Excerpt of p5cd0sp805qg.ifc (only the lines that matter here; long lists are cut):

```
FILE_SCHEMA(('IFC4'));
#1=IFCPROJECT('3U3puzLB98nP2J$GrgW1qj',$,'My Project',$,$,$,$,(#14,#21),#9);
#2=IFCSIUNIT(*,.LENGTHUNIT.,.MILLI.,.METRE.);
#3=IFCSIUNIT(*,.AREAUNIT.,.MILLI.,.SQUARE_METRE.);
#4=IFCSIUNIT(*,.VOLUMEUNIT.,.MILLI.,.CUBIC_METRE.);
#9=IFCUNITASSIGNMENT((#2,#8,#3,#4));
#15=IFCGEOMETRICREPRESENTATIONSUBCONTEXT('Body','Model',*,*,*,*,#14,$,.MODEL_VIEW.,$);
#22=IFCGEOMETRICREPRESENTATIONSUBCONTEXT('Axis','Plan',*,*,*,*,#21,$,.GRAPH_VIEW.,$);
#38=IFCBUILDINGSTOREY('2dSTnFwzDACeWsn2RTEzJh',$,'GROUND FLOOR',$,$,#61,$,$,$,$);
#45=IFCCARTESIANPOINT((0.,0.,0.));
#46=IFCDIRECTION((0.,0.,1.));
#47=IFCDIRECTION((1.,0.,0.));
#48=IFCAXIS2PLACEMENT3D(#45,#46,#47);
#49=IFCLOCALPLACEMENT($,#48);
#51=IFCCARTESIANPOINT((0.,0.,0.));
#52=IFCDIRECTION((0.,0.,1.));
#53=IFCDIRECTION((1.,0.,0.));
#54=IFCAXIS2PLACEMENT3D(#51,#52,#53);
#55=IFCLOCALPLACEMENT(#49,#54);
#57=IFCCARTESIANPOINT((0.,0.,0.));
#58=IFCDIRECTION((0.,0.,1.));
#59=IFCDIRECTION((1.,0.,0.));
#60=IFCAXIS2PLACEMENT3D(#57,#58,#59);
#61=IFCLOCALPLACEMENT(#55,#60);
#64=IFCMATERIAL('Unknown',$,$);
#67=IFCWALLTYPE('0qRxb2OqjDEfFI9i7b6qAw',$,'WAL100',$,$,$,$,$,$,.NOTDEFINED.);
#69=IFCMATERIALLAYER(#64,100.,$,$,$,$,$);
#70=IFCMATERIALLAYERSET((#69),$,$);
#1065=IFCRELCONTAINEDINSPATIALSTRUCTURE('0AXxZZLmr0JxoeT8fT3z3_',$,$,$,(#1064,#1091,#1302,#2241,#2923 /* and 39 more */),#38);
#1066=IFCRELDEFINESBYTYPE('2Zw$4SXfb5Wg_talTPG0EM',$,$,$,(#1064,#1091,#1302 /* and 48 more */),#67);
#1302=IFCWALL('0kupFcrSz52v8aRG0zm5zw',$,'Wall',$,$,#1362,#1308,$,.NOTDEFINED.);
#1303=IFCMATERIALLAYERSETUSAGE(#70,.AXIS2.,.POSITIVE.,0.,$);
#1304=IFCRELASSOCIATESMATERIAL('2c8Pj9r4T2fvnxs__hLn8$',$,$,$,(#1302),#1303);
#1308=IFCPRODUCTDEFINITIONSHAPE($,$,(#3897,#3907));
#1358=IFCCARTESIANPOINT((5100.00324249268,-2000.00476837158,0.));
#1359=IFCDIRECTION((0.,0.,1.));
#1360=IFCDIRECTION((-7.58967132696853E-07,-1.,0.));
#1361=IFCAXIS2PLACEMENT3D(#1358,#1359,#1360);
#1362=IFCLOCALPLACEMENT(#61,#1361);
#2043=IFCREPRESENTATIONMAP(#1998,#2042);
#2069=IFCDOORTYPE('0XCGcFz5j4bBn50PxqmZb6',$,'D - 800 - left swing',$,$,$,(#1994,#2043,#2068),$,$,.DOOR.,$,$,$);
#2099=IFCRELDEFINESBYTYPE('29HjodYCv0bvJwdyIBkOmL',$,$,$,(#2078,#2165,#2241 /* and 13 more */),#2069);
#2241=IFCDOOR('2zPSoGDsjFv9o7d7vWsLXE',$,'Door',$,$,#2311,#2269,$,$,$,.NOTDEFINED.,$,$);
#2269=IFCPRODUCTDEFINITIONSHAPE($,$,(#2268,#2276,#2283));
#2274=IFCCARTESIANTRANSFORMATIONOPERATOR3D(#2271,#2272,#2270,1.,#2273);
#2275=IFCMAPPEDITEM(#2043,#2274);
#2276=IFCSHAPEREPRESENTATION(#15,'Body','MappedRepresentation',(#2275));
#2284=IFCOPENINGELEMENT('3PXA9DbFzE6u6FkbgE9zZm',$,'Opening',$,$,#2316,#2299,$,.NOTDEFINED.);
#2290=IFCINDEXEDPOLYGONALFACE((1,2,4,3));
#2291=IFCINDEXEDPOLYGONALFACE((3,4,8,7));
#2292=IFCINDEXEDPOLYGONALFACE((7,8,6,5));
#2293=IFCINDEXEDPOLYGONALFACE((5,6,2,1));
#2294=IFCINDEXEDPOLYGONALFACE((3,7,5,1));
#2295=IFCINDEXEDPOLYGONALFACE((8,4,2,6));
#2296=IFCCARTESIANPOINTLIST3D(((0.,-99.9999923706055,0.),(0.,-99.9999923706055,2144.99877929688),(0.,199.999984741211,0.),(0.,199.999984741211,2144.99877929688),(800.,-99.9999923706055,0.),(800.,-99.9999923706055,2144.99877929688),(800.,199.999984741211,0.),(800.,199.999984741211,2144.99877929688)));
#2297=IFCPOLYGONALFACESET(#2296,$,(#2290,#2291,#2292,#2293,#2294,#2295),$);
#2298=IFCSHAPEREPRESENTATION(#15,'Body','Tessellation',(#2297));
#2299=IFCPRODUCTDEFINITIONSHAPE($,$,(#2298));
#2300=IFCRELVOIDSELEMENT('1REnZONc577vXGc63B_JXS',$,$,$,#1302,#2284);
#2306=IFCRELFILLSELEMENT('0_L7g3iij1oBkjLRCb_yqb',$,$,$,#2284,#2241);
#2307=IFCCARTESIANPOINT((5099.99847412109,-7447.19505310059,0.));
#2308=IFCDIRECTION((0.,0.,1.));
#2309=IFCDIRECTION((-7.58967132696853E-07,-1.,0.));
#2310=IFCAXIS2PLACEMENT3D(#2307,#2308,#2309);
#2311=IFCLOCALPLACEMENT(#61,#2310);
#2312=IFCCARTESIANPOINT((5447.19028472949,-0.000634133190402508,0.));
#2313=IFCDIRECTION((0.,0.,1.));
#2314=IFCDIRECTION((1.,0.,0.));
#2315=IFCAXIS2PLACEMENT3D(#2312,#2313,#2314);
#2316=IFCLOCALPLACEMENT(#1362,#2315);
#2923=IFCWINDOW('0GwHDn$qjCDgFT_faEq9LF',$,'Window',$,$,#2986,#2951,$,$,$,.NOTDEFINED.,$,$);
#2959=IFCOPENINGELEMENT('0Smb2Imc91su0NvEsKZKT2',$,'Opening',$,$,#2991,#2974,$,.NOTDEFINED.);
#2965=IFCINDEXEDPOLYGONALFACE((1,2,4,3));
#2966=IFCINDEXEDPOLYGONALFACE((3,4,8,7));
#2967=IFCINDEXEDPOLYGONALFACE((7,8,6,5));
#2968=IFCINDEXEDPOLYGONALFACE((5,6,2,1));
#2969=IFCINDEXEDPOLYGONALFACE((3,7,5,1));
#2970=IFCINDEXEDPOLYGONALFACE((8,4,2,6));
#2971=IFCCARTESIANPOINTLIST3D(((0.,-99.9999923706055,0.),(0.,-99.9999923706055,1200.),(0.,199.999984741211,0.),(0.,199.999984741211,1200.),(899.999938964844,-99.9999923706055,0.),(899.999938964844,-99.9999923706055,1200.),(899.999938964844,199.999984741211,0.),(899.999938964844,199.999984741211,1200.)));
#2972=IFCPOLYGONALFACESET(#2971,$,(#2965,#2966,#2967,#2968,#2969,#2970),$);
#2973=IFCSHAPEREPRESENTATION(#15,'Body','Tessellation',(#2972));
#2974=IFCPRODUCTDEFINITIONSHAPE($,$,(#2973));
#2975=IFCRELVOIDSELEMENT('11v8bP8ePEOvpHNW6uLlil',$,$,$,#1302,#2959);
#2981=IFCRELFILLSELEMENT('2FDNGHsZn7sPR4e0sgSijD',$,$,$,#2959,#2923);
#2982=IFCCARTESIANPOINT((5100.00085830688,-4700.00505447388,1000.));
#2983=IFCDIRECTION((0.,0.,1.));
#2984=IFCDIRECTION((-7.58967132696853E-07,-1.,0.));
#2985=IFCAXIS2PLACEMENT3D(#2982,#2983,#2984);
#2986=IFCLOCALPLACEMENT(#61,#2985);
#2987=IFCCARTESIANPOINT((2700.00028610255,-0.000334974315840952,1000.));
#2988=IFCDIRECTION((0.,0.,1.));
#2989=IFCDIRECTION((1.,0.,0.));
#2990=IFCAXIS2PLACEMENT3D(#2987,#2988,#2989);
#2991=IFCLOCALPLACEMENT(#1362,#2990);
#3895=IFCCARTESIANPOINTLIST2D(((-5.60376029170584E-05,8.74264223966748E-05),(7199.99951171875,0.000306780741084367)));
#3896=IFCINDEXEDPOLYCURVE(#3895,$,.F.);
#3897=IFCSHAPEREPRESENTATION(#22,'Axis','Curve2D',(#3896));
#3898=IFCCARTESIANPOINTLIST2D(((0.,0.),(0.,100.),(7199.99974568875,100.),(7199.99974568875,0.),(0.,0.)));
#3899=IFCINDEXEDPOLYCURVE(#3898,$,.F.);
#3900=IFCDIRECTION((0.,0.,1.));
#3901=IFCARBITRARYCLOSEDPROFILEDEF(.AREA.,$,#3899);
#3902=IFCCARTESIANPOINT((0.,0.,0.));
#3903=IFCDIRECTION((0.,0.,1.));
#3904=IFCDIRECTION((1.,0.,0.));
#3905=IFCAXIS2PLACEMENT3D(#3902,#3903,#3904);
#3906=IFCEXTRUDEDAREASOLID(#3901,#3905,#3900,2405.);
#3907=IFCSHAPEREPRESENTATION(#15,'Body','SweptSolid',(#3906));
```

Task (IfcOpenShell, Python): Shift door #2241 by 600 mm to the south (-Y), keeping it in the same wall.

```python
import ifcopenshell
import ifcopenshell.api.geometry
import ifcopenshell.util.placement
import ifcopenshell.util.unit

model = ifcopenshell.open("p5cd0sp805qg.ifc")
unit_scale = ifcopenshell.util.unit.calculate_unit_scale(model)

door = model.by_guid("2zPSoGDsjFv9o7d7vWsLXE")
opening = door.FillsVoids[0].RelatingOpeningElement
wall = opening.VoidsElements[0].RelatingBuildingElement

wall_matrix = ifcopenshell.util.placement.get_local_placement(wall.ObjectPlacement)
shift = wall_matrix[:3, 0] * 0.6 / unit_scale
before = ifcopenshell.util.placement.get_local_placement(door.ObjectPlacement)[:3, 3].copy()

# The door is not placed relative to its opening, so move both.
for product in (opening, door):
    matrix = ifcopenshell.util.placement.get_local_placement(product.ObjectPlacement)
    matrix[:3, 3] += shift
    ifcopenshell.api.geometry.edit_object_placement(model, product=product, matrix=matrix, is_si=False)

after = ifcopenshell.util.placement.get_local_placement(door.ObjectPlacement)[:3, 3]
print("door moved by", (after - before).round(3) + 0.0)

model.write("p5cd0sp805qg_edited.ifc")
```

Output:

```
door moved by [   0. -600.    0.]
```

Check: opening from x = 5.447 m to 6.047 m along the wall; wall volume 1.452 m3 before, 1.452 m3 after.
